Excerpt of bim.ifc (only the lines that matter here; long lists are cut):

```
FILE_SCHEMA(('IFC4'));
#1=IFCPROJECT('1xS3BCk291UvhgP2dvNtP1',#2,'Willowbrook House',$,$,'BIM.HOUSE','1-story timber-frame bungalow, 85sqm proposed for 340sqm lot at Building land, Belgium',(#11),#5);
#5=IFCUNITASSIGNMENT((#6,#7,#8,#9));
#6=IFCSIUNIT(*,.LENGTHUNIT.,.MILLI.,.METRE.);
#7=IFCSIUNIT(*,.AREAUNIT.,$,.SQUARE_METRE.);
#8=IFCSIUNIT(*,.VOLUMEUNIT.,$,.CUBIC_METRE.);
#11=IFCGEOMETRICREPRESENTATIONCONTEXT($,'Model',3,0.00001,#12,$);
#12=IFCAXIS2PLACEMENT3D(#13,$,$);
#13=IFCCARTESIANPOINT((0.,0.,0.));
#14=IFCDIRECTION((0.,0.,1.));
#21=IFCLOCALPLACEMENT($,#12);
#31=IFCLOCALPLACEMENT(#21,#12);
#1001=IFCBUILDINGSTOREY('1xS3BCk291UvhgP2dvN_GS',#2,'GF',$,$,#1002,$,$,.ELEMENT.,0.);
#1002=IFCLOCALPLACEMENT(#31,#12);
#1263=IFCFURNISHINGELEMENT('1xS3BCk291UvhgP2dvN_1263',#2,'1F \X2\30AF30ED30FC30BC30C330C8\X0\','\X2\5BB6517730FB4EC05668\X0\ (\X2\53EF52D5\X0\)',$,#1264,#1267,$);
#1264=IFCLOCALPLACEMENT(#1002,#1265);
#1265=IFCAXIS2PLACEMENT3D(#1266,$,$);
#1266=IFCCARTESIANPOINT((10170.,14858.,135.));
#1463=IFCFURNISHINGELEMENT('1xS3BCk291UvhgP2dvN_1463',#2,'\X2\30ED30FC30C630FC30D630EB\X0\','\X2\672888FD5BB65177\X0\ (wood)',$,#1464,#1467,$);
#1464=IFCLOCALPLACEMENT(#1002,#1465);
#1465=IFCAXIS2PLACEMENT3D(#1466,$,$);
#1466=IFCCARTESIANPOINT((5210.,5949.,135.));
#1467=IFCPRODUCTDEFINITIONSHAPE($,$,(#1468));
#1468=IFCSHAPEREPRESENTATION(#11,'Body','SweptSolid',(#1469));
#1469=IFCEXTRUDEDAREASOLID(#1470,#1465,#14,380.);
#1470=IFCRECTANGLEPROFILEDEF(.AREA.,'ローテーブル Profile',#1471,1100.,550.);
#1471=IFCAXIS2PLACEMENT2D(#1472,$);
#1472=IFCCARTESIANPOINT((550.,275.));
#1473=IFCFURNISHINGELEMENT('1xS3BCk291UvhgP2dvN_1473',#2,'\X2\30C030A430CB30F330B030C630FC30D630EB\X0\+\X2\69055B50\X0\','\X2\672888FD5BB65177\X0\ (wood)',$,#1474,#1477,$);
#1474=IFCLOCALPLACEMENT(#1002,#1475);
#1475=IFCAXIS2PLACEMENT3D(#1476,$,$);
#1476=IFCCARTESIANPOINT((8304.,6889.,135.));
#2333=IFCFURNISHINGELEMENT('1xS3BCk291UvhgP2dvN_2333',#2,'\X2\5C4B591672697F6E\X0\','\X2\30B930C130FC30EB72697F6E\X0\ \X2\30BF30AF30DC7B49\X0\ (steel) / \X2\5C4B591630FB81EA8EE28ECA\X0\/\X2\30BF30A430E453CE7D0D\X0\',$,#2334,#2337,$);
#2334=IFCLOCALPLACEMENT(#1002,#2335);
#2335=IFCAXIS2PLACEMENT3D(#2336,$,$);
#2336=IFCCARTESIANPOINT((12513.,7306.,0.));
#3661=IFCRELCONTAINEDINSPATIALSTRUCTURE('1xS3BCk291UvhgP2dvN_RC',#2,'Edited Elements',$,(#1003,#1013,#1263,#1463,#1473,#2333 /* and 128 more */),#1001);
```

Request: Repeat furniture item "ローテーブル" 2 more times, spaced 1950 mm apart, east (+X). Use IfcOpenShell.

```python
import numpy as np
import ifcopenshell
import ifcopenshell.api.geometry
import ifcopenshell.api.root
import ifcopenshell.util.element
import ifcopenshell.util.placement
import ifcopenshell.util.unit

model = ifcopenshell.open("bim.ifc")
unit_scale = ifcopenshell.util.unit.calculate_unit_scale(model)


def reuse_history(source, copy):
    """copy_class also copies each property set's owner history, people and application; keep the originals."""
    for rel in copy.IsDefinedBy:
        if rel.is_a("IfcRelDefinesByProperties") and (history := rel.RelatingPropertyDefinition.OwnerHistory):
            rel.RelatingPropertyDefinition.OwnerHistory = source.OwnerHistory
            ifcopenshell.util.element.remove_deep2(model, history)


source = model.by_guid("1xS3BCk291UvhgP2dvN_1463")
base = ifcopenshell.util.placement.get_local_placement(source.ObjectPlacement)
step = np.array([1.0, 0.0, 0.0]) * 1.95 / unit_scale

for i in range(1, 3):
    copy = ifcopenshell.api.root.copy_class(model, product=source)
    copy.Representation = ifcopenshell.util.element.copy_deep(
        model, source.Representation, exclude=["IfcGeometricRepresentationContext", "IfcRepresentationMap"]
    )
    reuse_history(source, copy)
    matrix = base.copy()
    matrix[:3, 3] += i * step
    print("added at", matrix[:3, 3].round(3) + 0.0)
    ifcopenshell.api.geometry.edit_object_placement(model, product=copy, matrix=matrix, is_si=False)

model.write("bim_updated.ifc")
```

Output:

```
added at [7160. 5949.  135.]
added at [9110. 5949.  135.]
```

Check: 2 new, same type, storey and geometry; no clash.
